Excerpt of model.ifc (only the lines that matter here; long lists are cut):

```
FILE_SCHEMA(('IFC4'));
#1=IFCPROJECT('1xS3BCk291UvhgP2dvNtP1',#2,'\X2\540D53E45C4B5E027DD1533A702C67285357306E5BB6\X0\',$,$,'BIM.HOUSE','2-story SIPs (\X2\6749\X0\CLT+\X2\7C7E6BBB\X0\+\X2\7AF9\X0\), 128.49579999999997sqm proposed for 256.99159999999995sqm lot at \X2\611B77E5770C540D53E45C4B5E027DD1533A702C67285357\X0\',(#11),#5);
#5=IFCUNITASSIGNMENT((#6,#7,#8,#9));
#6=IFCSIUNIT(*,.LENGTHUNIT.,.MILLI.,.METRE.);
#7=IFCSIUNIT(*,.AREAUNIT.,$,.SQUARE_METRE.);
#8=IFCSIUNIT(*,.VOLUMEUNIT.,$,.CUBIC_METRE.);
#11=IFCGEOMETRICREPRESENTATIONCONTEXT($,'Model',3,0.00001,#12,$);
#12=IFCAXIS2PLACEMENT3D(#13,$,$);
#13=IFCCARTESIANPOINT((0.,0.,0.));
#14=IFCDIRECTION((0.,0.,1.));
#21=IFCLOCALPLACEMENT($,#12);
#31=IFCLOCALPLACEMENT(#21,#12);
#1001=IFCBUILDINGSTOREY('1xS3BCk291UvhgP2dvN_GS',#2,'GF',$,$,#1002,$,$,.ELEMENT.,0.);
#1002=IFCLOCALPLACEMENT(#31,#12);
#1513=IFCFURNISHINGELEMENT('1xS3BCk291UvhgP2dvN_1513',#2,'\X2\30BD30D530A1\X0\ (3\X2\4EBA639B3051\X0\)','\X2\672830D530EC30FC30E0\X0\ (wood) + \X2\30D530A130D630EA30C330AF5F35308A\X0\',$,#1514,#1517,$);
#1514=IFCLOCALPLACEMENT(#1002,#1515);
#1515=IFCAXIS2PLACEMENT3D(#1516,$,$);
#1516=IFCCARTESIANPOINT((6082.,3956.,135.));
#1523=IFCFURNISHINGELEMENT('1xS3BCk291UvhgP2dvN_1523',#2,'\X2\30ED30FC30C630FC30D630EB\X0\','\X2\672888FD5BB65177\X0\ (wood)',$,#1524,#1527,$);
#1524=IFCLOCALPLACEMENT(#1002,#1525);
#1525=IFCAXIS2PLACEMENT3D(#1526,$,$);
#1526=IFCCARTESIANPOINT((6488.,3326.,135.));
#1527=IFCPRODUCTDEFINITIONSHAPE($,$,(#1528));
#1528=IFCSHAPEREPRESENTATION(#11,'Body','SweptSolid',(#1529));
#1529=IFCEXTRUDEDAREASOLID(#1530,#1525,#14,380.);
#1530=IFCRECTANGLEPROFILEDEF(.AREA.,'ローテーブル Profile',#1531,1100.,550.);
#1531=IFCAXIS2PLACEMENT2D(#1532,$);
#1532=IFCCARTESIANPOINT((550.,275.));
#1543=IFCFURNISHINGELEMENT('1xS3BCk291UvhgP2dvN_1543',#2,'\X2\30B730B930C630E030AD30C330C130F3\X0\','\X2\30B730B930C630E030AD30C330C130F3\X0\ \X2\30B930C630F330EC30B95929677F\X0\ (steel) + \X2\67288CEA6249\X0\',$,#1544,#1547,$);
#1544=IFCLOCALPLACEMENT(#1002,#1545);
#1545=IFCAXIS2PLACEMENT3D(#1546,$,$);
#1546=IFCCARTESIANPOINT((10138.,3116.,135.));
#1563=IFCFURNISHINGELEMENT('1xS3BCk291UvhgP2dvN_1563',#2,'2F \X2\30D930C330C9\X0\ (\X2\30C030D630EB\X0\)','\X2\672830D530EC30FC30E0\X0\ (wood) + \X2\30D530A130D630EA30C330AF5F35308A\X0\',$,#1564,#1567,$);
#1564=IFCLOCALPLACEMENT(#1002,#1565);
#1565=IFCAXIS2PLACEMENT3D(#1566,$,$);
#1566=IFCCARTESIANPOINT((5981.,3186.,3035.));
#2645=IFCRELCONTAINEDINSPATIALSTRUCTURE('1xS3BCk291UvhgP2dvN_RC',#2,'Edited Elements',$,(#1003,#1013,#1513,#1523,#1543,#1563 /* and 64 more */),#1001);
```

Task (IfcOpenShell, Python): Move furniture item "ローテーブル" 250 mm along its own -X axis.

```python
import ifcopenshell
import ifcopenshell.api.geometry
import ifcopenshell.util.placement
import ifcopenshell.util.unit

model = ifcopenshell.open("model.ifc")
unit_scale = ifcopenshell.util.unit.calculate_unit_scale(model)

item = model.by_guid("1xS3BCk291UvhgP2dvN_1523")
matrix = ifcopenshell.util.placement.get_local_placement(item.ObjectPlacement)
matrix[:3, 3] -= matrix[:3, 0] * 0.25 / unit_scale
ifcopenshell.api.geometry.edit_object_placement(model, product=item, matrix=matrix, is_si=False)

print(ifcopenshell.util.placement.get_local_placement(item.ObjectPlacement).round(3) + 0.0)

model.write("model_updated.ifc")
```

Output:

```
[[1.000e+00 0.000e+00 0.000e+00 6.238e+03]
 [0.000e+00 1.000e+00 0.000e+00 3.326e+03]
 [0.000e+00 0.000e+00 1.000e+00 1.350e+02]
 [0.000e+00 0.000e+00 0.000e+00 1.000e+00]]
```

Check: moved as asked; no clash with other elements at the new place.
